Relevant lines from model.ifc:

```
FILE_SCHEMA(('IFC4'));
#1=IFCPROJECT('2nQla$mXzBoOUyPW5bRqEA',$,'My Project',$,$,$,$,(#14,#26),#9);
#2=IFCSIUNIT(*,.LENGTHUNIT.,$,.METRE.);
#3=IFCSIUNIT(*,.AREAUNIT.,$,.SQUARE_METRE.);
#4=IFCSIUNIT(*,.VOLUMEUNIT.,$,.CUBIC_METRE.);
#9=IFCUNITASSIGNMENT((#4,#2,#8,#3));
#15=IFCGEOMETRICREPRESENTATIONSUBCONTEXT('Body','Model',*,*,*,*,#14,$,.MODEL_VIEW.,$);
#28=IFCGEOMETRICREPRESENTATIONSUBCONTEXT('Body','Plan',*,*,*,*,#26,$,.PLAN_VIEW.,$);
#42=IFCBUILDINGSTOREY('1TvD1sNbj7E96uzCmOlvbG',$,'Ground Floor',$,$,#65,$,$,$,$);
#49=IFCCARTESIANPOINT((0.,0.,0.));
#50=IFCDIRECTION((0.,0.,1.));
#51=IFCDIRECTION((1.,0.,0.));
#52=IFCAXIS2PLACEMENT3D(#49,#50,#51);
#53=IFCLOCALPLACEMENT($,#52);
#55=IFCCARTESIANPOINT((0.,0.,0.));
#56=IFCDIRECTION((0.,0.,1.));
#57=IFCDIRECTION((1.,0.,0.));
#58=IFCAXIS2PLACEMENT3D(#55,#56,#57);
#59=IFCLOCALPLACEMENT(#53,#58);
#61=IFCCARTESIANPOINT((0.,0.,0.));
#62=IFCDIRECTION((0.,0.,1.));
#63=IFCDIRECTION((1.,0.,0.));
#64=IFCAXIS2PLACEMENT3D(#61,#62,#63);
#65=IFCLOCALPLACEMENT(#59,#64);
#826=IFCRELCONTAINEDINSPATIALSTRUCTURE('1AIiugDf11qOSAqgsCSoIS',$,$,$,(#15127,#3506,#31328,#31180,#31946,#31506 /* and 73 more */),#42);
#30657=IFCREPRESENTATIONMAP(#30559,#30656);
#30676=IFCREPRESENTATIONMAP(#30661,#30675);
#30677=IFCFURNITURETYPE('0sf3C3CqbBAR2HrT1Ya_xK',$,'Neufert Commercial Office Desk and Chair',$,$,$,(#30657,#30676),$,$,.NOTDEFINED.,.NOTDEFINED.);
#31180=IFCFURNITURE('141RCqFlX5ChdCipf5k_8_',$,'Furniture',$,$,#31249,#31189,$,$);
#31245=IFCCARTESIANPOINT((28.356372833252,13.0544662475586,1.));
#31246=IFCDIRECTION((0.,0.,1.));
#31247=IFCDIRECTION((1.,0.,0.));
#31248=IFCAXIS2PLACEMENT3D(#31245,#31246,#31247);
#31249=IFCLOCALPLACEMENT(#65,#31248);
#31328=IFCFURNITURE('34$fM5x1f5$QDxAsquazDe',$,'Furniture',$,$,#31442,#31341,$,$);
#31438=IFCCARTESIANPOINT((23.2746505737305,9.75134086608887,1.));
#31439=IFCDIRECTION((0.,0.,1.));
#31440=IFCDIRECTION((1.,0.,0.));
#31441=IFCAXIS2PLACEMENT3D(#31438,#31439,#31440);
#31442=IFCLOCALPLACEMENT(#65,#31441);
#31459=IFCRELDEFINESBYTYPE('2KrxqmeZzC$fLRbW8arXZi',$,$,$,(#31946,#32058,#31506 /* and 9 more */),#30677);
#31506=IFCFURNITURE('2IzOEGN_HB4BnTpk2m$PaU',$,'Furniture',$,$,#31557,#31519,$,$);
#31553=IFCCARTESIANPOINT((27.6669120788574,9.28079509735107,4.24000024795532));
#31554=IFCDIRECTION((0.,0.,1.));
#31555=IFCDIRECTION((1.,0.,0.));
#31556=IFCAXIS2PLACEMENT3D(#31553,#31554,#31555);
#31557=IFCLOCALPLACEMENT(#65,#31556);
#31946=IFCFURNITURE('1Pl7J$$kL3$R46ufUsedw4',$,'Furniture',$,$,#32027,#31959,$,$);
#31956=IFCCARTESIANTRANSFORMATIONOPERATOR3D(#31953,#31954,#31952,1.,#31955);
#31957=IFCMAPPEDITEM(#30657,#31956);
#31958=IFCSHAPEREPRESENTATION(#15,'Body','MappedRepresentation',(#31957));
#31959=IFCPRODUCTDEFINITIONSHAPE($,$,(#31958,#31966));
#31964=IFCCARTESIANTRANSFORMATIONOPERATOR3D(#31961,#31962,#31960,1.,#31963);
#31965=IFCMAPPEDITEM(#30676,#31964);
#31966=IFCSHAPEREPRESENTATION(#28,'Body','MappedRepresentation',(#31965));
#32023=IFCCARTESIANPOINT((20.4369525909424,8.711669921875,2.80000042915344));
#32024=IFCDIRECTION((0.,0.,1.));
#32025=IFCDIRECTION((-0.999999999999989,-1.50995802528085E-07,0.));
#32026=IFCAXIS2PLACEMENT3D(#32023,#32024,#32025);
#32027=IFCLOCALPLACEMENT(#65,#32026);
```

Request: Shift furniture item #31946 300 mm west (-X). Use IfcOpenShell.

```python
import ifcopenshell
import ifcopenshell.api.geometry
import ifcopenshell.util.placement
import ifcopenshell.util.unit

model = ifcopenshell.open("model.ifc")
unit_scale = ifcopenshell.util.unit.calculate_unit_scale(model)

item = model.by_guid("1Pl7J$$kL3$R46ufUsedw4")
matrix = ifcopenshell.util.placement.get_local_placement(item.ObjectPlacement)
matrix[0, 3] -= 0.3 / unit_scale
ifcopenshell.api.geometry.edit_object_placement(model, product=item, matrix=matrix, is_si=False)

print(ifcopenshell.util.placement.get_local_placement(item.ObjectPlacement).round(3) + 0.0)

model.write("model_rev.ifc")
```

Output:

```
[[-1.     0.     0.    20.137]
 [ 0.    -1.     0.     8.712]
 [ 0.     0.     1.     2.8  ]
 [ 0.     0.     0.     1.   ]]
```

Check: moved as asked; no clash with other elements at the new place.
